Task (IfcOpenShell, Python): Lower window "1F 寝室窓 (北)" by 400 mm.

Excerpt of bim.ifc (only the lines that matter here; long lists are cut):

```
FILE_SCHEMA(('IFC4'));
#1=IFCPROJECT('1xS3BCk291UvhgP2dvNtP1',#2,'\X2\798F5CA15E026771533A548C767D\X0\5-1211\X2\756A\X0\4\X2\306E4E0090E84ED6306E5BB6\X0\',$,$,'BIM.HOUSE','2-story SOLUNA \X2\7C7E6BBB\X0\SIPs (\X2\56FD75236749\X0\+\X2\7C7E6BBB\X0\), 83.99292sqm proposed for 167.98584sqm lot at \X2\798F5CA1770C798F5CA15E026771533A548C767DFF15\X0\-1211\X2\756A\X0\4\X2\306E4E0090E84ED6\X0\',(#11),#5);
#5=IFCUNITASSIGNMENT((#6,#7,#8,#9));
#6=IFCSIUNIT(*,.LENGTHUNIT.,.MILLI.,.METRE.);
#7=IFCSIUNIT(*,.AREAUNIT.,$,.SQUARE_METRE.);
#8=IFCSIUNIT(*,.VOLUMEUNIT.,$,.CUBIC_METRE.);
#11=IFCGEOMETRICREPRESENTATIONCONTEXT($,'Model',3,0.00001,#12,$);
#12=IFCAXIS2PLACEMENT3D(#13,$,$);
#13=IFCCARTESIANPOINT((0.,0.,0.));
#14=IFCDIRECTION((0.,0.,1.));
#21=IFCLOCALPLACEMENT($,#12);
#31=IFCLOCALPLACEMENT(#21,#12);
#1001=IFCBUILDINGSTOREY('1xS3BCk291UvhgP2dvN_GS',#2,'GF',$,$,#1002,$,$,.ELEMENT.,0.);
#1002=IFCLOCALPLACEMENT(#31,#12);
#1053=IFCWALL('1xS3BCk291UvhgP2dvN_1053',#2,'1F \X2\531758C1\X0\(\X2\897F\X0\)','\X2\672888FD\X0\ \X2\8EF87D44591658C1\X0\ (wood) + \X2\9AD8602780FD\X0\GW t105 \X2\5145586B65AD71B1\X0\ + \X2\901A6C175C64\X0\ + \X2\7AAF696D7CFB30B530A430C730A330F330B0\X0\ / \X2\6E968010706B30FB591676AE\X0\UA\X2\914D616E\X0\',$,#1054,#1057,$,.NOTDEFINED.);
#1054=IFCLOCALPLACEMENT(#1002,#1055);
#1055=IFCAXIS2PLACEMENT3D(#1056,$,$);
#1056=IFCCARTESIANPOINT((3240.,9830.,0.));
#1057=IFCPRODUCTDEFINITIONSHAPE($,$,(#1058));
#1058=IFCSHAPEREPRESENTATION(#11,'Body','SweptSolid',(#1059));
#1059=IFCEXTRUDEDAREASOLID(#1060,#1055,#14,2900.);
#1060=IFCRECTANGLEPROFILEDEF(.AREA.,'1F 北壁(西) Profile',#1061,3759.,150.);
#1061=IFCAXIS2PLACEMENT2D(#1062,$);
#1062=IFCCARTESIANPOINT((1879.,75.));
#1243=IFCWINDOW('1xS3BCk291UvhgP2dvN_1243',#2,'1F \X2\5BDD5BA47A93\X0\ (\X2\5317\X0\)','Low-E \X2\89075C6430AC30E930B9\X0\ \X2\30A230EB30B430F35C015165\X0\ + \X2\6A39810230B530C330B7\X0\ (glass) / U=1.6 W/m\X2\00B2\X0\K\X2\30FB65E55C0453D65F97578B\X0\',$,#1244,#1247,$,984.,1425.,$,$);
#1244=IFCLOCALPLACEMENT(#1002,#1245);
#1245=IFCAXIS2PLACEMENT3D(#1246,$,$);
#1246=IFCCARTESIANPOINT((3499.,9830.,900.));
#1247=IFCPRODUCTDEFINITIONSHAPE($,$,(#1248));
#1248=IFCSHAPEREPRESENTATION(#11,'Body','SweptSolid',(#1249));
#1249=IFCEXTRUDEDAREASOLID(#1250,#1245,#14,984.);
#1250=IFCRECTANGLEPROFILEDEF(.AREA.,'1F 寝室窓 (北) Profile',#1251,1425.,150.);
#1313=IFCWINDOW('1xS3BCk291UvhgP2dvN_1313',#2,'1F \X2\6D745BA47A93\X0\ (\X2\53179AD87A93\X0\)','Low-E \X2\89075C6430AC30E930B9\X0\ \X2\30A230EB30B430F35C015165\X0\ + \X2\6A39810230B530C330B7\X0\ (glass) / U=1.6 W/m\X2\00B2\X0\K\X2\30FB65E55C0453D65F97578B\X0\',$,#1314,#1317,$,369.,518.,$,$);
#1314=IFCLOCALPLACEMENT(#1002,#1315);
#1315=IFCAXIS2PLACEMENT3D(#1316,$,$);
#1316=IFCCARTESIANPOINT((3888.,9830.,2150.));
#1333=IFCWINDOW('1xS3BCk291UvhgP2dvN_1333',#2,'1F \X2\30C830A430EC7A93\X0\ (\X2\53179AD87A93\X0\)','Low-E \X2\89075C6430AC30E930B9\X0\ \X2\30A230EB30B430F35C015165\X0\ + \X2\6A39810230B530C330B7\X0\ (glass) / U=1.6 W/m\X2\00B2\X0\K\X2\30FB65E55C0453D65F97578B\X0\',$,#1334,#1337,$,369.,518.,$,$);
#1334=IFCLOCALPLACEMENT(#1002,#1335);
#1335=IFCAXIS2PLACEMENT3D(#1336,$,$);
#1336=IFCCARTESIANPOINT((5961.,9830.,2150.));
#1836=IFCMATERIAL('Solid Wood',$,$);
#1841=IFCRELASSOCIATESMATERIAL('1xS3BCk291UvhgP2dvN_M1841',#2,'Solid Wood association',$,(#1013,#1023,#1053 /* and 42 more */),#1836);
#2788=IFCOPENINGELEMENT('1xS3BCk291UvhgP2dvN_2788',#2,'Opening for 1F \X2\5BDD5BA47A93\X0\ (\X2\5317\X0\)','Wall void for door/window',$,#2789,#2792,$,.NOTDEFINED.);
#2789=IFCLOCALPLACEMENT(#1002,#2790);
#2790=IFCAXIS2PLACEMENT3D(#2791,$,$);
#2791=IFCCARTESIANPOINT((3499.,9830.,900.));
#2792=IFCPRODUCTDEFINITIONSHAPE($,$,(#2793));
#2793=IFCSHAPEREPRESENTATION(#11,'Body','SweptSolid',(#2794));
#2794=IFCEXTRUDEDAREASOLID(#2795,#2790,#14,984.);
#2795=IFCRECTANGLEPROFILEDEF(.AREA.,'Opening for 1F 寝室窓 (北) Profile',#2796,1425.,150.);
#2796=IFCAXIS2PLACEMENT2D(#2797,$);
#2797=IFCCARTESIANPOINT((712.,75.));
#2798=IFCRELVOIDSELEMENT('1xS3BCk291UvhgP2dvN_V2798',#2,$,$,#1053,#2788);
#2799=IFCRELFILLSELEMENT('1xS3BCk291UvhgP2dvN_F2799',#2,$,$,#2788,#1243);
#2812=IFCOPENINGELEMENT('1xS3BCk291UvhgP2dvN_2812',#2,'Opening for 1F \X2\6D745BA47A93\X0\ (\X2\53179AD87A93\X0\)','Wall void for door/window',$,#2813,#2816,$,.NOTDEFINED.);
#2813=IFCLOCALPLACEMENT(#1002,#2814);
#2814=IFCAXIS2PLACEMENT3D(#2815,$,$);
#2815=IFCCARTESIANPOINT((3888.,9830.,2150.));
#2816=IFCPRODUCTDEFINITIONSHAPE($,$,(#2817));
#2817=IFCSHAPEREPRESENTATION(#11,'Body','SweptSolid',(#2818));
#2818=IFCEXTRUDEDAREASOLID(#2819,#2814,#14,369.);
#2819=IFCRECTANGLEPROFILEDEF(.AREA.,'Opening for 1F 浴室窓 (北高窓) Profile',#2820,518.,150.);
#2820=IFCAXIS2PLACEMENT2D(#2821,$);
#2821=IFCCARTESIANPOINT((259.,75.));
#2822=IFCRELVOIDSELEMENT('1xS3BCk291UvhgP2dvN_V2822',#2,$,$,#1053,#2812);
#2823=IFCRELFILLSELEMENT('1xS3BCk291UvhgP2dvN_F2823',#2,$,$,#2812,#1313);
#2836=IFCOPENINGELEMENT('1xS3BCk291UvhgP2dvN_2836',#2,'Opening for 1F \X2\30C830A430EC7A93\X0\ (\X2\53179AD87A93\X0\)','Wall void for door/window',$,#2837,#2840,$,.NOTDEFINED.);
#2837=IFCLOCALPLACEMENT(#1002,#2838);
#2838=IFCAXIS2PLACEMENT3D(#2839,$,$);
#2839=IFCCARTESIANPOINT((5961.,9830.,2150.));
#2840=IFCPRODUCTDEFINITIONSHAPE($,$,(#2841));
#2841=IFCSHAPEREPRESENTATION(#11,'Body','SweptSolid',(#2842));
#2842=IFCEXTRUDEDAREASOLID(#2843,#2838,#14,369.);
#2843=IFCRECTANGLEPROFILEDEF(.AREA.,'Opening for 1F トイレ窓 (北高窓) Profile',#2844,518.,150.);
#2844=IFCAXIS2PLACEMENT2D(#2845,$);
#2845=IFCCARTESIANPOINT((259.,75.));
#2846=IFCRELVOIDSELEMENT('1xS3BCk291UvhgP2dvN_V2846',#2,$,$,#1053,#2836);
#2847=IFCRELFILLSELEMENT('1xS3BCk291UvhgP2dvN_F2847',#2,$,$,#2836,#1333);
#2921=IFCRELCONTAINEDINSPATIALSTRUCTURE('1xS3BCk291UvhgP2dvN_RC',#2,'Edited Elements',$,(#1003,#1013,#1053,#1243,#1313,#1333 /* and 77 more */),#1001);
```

```python
import numpy as np
import ifcopenshell
import ifcopenshell.api.geometry
import ifcopenshell.util.placement
import ifcopenshell.util.unit

model = ifcopenshell.open("bim.ifc")
unit_scale = ifcopenshell.util.unit.calculate_unit_scale(model)

window = model.by_guid("1xS3BCk291UvhgP2dvN_1243")
opening = window.FillsVoids[0].RelatingOpeningElement
dz = -400.0

shift = np.array([0.0, 0.0, dz])
# The window is not placed relative to its opening, so move both.
for product in (opening, window):
    matrix = ifcopenshell.util.placement.get_local_placement(product.ObjectPlacement)
    matrix[:3, 3] += shift
    ifcopenshell.api.geometry.edit_object_placement(model, product=product, matrix=matrix, is_si=False)

print(f"moved by {dz * unit_scale:+.3f} m")

model.write("bim_rev.ifc")
```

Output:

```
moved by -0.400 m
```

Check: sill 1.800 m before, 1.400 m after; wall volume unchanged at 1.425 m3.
